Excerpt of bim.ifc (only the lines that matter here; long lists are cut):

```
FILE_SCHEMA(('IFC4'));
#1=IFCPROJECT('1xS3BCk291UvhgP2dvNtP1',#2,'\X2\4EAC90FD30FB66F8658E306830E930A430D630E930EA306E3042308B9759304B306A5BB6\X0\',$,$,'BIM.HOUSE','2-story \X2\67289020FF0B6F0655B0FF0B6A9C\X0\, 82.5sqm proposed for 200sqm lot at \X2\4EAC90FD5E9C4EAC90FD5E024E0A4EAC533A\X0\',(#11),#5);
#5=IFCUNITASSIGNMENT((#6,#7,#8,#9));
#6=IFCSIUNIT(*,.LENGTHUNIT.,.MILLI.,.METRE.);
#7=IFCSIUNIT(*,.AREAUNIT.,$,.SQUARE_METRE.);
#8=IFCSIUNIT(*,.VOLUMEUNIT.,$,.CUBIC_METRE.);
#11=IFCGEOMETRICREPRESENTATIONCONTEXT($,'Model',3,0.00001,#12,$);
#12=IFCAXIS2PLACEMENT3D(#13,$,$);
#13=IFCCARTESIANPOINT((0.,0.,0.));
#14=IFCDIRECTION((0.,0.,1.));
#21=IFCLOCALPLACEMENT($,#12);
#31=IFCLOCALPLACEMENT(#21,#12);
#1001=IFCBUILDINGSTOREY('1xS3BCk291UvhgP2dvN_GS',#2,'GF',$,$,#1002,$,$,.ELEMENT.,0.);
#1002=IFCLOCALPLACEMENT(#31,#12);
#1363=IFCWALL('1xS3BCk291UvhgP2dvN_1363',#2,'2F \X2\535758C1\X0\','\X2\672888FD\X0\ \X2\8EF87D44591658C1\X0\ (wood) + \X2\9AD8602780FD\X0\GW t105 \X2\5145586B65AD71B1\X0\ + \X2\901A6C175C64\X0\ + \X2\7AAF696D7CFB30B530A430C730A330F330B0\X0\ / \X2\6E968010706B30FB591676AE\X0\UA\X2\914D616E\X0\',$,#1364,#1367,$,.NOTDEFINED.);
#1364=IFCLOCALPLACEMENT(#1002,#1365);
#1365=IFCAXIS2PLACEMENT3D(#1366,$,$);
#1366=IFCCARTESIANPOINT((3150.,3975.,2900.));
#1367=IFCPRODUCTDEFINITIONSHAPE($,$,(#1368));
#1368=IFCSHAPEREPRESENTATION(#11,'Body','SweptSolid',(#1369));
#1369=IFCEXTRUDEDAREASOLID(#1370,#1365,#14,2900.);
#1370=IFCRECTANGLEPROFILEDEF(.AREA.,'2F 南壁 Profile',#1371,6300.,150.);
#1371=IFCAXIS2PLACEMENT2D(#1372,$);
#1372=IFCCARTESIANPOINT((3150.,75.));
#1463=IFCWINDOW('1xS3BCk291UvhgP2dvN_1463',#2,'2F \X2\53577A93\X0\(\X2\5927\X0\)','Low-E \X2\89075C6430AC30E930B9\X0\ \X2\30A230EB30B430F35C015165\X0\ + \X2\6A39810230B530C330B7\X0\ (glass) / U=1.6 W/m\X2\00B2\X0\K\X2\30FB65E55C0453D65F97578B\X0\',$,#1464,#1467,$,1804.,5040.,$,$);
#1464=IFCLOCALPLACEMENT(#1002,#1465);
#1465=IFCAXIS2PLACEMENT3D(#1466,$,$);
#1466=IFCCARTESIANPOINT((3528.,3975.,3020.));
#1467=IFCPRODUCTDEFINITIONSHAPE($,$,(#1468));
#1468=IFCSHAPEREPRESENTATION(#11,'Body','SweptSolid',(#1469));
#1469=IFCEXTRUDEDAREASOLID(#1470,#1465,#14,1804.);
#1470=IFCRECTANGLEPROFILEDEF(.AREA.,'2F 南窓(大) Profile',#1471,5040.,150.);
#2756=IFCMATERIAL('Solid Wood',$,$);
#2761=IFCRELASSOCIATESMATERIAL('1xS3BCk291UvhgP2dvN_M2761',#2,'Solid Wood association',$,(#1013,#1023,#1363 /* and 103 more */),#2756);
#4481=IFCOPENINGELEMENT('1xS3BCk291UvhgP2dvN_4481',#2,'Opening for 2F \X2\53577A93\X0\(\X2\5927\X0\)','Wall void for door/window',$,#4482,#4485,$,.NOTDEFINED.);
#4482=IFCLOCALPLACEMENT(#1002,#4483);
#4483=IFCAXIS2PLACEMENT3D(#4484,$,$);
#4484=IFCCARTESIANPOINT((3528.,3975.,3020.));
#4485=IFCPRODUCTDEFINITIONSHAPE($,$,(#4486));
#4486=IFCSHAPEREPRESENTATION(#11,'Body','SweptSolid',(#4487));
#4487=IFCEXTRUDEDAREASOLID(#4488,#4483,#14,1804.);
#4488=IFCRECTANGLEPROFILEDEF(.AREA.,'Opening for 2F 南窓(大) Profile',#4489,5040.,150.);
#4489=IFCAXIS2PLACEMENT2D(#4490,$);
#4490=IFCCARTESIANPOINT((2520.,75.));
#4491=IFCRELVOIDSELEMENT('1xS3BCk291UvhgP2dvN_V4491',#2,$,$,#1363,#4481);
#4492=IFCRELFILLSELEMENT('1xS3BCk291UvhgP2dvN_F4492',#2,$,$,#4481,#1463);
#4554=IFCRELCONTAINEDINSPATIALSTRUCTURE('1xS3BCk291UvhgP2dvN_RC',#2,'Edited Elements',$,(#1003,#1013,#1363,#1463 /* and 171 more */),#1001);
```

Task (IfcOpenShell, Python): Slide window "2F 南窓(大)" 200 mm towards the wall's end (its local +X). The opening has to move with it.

```python
import ifcopenshell
import ifcopenshell.api.geometry
import ifcopenshell.util.placement
import ifcopenshell.util.unit

model = ifcopenshell.open("bim.ifc")
unit_scale = ifcopenshell.util.unit.calculate_unit_scale(model)

window = model.by_id(1463)
opening = window.FillsVoids[0].RelatingOpeningElement
wall = opening.VoidsElements[0].RelatingBuildingElement

wall_matrix = ifcopenshell.util.placement.get_local_placement(wall.ObjectPlacement)
shift = wall_matrix[:3, 0] * 0.2 / unit_scale
before = ifcopenshell.util.placement.get_local_placement(window.ObjectPlacement)[:3, 3].copy()

# The window is not placed relative to its opening, so move both.
for product in (opening, window):
    matrix = ifcopenshell.util.placement.get_local_placement(product.ObjectPlacement)
    matrix[:3, 3] += shift
    ifcopenshell.api.geometry.edit_object_placement(model, product=product, matrix=matrix, is_si=False)

after = ifcopenshell.util.placement.get_local_placement(window.ObjectPlacement)[:3, 3]
print("window moved by", (after - before).round(3) + 0.0)

model.write("bim-out.ifc")
```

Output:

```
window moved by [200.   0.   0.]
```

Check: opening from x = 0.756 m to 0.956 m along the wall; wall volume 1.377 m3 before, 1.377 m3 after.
